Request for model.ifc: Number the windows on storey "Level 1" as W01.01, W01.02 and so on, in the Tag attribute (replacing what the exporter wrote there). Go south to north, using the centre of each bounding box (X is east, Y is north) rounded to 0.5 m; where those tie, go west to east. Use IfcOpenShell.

First a look at what the model holds.

```python
import ifcopenshell
import ifcopenshell.util.element
import ifcopenshell.util.placement

model = ifcopenshell.open("model.ifc")
print(model.schema)
storey = next(s for s in model.by_type("IfcBuildingStorey") if s.Name == "Level 1")
windows = [e for e in ifcopenshell.util.element.get_decomposition(storey) if e.is_a("IfcWindow")]
for e in sorted(windows, key=lambda e: e.id()):
    origin = ifcopenshell.util.placement.get_local_placement(e.ObjectPlacement)[:3, 3]
    print(e.id(), e.Tag, e.Name, origin.round(2) + 0.0, sep=" | ")
```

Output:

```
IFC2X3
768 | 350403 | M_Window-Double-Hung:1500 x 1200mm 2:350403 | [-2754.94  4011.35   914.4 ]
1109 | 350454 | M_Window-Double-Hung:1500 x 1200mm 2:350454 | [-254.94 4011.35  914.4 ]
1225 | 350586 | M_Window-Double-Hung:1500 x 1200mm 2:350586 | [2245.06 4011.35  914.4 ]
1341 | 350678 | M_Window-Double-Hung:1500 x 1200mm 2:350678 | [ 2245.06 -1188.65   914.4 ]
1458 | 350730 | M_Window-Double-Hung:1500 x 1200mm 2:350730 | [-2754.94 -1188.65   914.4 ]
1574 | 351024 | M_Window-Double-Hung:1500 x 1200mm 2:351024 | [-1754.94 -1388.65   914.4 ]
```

```python
import ifcopenshell
import ifcopenshell.geom
import ifcopenshell.util.element
import ifcopenshell.util.shape

model = ifcopenshell.open("model.ifc")
settings = ifcopenshell.geom.settings()
settings.set("use-world-coords", True)


def centre(element):
    shape = ifcopenshell.geom.create_shape(settings, element)
    return ifcopenshell.util.shape.get_bbox_centroid(shape.geometry)


storey = next(s for s in model.by_type("IfcBuildingStorey") if s.Name == "Level 1")
windows = [e for e in ifcopenshell.util.element.get_decomposition(storey) if e.is_a("IfcWindow")]

# Insertion points can sit at a corner or the storey origin, so sort by the geometry (in metres).
centres = {e: centre(e) for e in windows}
windows.sort(key=lambda e: (round(centres[e][1] / 0.5), centres[e][0]))

for i, e in enumerate(windows, start=1):
    number = f"W01.{i:02d}"
    e.Tag = number
    print(e.id(), number)

model.write("model_rev.ifc")
```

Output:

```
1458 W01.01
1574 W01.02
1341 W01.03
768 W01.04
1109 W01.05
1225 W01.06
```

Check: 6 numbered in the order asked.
